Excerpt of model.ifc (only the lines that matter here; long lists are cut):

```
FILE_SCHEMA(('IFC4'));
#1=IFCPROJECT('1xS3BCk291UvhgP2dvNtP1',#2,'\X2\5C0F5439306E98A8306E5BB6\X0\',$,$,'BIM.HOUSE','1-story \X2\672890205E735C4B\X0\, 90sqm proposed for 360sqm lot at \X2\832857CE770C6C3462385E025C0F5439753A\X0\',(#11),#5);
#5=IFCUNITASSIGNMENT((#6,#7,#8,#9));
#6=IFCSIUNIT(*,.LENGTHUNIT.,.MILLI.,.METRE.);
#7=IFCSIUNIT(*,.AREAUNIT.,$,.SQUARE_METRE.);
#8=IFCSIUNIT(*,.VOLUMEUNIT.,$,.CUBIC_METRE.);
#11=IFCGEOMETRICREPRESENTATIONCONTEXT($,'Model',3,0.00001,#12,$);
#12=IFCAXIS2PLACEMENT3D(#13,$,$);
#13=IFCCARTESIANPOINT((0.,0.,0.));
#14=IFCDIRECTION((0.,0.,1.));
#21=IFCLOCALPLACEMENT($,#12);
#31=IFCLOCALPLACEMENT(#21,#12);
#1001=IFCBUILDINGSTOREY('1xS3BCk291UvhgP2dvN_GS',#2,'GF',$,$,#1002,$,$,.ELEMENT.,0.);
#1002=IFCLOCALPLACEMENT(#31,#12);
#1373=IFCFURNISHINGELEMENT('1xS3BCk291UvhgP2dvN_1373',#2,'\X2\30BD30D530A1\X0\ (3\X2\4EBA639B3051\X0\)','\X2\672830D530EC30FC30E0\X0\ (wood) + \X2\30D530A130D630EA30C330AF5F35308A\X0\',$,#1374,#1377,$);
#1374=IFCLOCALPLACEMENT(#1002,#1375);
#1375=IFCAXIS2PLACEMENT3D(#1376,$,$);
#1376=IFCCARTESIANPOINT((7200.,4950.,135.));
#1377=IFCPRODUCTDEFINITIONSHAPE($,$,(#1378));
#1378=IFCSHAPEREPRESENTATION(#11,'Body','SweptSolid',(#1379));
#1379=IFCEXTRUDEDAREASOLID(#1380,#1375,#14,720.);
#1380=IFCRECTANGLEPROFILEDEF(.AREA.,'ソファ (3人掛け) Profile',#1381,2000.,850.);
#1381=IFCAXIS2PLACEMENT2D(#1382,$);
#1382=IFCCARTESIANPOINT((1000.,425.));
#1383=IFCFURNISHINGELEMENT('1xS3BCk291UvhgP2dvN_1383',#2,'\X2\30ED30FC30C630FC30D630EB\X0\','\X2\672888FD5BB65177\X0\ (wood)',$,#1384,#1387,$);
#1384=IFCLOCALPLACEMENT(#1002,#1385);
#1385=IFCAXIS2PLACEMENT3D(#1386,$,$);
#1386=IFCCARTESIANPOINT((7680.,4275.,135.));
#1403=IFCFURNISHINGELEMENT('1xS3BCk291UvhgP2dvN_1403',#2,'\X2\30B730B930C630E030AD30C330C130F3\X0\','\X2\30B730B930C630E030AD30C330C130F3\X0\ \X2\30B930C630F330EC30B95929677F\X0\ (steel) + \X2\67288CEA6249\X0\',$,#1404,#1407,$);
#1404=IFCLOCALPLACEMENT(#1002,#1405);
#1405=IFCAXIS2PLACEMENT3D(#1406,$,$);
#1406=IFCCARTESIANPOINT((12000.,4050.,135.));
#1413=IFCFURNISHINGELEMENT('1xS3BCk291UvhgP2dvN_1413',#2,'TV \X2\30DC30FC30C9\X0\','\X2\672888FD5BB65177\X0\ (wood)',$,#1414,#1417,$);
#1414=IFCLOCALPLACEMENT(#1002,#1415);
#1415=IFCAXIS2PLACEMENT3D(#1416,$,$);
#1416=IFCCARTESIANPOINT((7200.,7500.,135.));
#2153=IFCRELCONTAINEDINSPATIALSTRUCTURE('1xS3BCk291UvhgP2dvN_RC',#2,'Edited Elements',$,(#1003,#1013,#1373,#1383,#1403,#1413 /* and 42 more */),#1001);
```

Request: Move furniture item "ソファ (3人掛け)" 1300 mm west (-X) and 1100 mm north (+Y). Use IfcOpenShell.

```python
import ifcopenshell
import ifcopenshell.api.geometry
import ifcopenshell.util.placement

model = ifcopenshell.open("model.ifc")

item = model.by_id(1373)
matrix = ifcopenshell.util.placement.get_local_placement(item.ObjectPlacement)
matrix[0, 3] -= 1300.0
matrix[1, 3] += 1100.0
ifcopenshell.api.geometry.edit_object_placement(model, product=item, matrix=matrix, is_si=False)

print(ifcopenshell.util.placement.get_local_placement(item.ObjectPlacement).round(3) + 0.0)

model.write("model_updated.ifc")
```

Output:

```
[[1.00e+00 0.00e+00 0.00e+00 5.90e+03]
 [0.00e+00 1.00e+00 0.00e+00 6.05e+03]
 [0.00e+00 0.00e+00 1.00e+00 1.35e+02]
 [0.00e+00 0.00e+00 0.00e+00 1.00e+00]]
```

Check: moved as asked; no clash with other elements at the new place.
